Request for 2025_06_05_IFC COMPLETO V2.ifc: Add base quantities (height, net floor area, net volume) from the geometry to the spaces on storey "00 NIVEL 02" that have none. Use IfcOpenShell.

First a look at what the model holds.

```python
import ifcopenshell
import ifcopenshell.util.element
import ifcopenshell.util.unit

model = ifcopenshell.open("2025_06_05_IFC COMPLETO V2.ifc")
print(model.schema)
for unit_type in ("LENGTHUNIT", "AREAUNIT", "VOLUMEUNIT"):
    print(unit_type, ifcopenshell.util.unit.calculate_unit_scale(model, unit_type))
storey = next(s for s in model.by_type("IfcBuildingStorey") if s.Name == "00 NIVEL 02")
spaces = [e for e in ifcopenshell.util.element.get_decomposition(storey) if e.is_a("IfcSpace")]
for e in sorted(spaces, key=lambda e: e.id()):
    print(e.id(), e.is_a(), e.Name, list(ifcopenshell.util.element.get_psets(e, qtos_only=True)), sep=" | ")
```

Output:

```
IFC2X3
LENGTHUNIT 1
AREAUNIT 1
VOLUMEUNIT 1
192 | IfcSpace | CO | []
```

```python
import ifcopenshell
import ifcopenshell.api.pset
import ifcopenshell.geom
import ifcopenshell.util.element
import ifcopenshell.util.shape
import ifcopenshell.util.unit

model = ifcopenshell.open("2025_06_05_IFC COMPLETO V2.ifc")
unit_scale = ifcopenshell.util.unit.calculate_unit_scale(model)
area_scale = ifcopenshell.util.unit.calculate_unit_scale(model, "AREAUNIT")
volume_scale = ifcopenshell.util.unit.calculate_unit_scale(model, "VOLUMEUNIT")
settings = ifcopenshell.geom.settings()

storey = next(s for s in model.by_type("IfcBuildingStorey") if s.Name == "00 NIVEL 02")
spaces = [e for e in ifcopenshell.util.element.get_decomposition(storey) if e.is_a("IfcSpace")]

for e in sorted(spaces, key=lambda e: e.id()):
    if ifcopenshell.util.element.get_psets(e, qtos_only=True, should_inherit=False):
        continue
    # Geometry comes back in metres, in the element's own axes.
    shape = ifcopenshell.geom.create_shape(settings, e)
    values = {
        "Height": ifcopenshell.util.shape.get_z(shape.geometry) / unit_scale,
        "NetFloorArea": ifcopenshell.util.shape.get_footprint_area(shape.geometry) / area_scale,
        "NetVolume": ifcopenshell.util.shape.get_volume(shape.geometry) / volume_scale,
    }
    qto = ifcopenshell.api.pset.add_qto(model, product=e, name="BaseQuantities")
    ifcopenshell.api.pset.edit_qto(model, qto=qto, properties=values)
    print(e.id(), {k: round(v, 3) for k, v in values.items()})

model.write("2025_06_05_IFC COMPLETO V2_v2.ifc")
```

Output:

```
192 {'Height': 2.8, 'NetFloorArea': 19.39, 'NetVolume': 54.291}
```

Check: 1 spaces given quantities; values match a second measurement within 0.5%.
